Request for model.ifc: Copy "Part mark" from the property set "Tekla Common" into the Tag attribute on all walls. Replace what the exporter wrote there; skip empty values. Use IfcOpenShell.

First a look at what the model holds.

```python
import ifcopenshell
import ifcopenshell.util.element

model = ifcopenshell.open("model.ifc")
print(model.schema)
walls = model.by_type("IfcWall")
print(len(walls), "walls")
for e in walls[:8]:
    source = ifcopenshell.util.element.get_pset(e, "Tekla Common", "Part mark")
    target = e.Tag
    print(e.id(), repr(source), repr(target), sep=" | ")
```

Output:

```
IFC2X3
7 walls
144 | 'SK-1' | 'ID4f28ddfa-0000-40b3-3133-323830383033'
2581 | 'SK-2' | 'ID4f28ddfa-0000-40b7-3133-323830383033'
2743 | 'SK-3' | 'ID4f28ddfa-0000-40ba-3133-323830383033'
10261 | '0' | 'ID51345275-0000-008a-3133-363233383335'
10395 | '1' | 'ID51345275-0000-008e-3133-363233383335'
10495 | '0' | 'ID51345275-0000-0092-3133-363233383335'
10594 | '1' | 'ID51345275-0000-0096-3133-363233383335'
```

```python
import ifcopenshell
import ifcopenshell.util.element

model = ifcopenshell.open("model.ifc")

count = 0
for e in model.by_type("IfcWall"):
    value = ifcopenshell.util.element.get_pset(e, "Tekla Common", "Part mark")
    current = e.Tag
    if not value or not value.strip() or current == value:
        continue
    e.Tag = value
    count += 1

print(count, "walls updated")

model.write("model_edited.ifc")
```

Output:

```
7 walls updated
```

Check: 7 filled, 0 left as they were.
